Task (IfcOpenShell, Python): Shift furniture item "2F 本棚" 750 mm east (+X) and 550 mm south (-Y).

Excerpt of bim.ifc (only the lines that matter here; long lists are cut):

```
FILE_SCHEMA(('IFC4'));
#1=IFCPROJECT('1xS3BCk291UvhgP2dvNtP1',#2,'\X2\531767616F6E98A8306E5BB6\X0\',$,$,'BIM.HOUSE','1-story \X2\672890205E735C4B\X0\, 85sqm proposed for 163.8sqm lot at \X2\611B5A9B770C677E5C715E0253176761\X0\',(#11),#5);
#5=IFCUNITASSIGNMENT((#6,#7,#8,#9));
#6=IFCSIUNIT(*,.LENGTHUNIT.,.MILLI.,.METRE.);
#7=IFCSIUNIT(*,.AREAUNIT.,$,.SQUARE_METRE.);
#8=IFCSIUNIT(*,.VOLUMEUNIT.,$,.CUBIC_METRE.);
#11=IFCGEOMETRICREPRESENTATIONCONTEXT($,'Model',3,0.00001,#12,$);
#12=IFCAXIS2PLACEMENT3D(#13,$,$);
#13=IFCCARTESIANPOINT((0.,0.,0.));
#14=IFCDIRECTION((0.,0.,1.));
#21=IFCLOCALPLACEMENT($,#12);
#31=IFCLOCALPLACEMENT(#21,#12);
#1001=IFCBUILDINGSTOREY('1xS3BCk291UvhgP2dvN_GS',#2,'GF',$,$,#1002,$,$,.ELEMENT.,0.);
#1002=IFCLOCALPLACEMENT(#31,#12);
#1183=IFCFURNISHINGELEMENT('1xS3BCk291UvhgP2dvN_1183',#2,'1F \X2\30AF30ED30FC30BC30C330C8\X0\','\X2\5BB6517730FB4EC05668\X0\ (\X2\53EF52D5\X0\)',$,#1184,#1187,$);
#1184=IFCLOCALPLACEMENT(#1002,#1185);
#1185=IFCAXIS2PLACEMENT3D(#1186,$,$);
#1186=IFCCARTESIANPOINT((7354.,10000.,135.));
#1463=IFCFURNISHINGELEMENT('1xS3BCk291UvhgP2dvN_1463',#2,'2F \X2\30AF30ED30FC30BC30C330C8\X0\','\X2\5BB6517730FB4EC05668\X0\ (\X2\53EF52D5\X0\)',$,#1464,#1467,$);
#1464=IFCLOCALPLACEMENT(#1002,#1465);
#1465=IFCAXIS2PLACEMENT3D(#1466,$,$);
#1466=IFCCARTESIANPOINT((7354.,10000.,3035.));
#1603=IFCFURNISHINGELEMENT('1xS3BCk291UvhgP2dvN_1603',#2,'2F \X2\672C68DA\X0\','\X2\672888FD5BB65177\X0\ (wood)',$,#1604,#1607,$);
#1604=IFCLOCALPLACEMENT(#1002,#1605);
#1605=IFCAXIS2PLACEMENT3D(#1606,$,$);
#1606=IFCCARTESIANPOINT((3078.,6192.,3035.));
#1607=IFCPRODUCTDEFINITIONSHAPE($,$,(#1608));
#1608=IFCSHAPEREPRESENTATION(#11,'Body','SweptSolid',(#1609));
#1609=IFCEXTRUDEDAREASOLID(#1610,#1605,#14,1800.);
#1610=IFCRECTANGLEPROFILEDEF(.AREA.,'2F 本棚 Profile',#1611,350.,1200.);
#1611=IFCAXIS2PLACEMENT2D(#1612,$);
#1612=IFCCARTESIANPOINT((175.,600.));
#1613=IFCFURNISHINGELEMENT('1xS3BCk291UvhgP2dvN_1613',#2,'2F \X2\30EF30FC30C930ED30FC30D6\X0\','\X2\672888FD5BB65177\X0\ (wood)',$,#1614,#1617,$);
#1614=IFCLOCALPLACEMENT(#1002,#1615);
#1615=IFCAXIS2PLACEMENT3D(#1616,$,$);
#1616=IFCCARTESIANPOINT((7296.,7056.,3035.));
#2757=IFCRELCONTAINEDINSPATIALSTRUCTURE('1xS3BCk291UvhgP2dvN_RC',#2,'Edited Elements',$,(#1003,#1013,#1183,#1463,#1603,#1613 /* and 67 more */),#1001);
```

```python
import ifcopenshell
import ifcopenshell.api.geometry
import ifcopenshell.util.placement

model = ifcopenshell.open("bim.ifc")

item = model.by_guid("1xS3BCk291UvhgP2dvN_1603")
matrix = ifcopenshell.util.placement.get_local_placement(item.ObjectPlacement)
matrix[0, 3] += 750.0
matrix[1, 3] -= 550.0
ifcopenshell.api.geometry.edit_object_placement(model, product=item, matrix=matrix, is_si=False)

print(ifcopenshell.util.placement.get_local_placement(item.ObjectPlacement).round(3) + 0.0)

model.write("bim-out.ifc")
```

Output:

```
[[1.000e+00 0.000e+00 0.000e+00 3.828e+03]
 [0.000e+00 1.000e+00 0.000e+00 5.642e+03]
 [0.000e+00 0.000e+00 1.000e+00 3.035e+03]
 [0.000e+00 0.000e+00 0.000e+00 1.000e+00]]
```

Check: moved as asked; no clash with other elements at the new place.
